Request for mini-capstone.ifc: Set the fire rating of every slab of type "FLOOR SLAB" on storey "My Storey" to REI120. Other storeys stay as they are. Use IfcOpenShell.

First a look at what the model holds.

```python
import ifcopenshell
import ifcopenshell.util.element

model = ifcopenshell.open("mini-capstone.ifc")
print(model.schema)
storey = next(s for s in model.by_type("IfcBuildingStorey") if s.Name == "My Storey")
slabs = [e for e in ifcopenshell.util.element.get_decomposition(storey) if e.is_a("IfcSlab")]
seen = {}
for e in slabs:
    element_type = ifcopenshell.util.element.get_type(e)
    key = (element_type.Name if element_type != e and element_type else None, ifcopenshell.util.element.get_pset(e, "Pset_SlabCommon", "FireRating"))
    seen[key] = seen.get(key, 0) + 1
for (name, value), count in sorted(seen.items(), key=str):
    print(count, "x", name, "|", value)
```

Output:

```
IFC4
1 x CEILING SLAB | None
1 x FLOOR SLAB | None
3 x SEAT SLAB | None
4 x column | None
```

```python
import ifcopenshell
import ifcopenshell.api.pset
import ifcopenshell.util.element

model = ifcopenshell.open("mini-capstone.ifc")

storey = next(s for s in model.by_type("IfcBuildingStorey") if s.Name == "My Storey")
slabs = [e for e in ifcopenshell.util.element.get_decomposition(storey) if e.is_a("IfcSlab")]

count = 0
for e in slabs:
    element_type = ifcopenshell.util.element.get_type(e)
    if element_type in (None, e) or element_type.Name != "FLOOR SLAB":
        continue
    # add_pset returns the element's existing set when there is one.
    pset = ifcopenshell.api.pset.add_pset(model, product=e, name="Pset_SlabCommon")
    ifcopenshell.api.pset.edit_pset(model, pset=pset, properties={"FireRating": "REI120"})
    count += 1

print(count, "slabs updated")

model.write("mini-capstone-out.ifc")
```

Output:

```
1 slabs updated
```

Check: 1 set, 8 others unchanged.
